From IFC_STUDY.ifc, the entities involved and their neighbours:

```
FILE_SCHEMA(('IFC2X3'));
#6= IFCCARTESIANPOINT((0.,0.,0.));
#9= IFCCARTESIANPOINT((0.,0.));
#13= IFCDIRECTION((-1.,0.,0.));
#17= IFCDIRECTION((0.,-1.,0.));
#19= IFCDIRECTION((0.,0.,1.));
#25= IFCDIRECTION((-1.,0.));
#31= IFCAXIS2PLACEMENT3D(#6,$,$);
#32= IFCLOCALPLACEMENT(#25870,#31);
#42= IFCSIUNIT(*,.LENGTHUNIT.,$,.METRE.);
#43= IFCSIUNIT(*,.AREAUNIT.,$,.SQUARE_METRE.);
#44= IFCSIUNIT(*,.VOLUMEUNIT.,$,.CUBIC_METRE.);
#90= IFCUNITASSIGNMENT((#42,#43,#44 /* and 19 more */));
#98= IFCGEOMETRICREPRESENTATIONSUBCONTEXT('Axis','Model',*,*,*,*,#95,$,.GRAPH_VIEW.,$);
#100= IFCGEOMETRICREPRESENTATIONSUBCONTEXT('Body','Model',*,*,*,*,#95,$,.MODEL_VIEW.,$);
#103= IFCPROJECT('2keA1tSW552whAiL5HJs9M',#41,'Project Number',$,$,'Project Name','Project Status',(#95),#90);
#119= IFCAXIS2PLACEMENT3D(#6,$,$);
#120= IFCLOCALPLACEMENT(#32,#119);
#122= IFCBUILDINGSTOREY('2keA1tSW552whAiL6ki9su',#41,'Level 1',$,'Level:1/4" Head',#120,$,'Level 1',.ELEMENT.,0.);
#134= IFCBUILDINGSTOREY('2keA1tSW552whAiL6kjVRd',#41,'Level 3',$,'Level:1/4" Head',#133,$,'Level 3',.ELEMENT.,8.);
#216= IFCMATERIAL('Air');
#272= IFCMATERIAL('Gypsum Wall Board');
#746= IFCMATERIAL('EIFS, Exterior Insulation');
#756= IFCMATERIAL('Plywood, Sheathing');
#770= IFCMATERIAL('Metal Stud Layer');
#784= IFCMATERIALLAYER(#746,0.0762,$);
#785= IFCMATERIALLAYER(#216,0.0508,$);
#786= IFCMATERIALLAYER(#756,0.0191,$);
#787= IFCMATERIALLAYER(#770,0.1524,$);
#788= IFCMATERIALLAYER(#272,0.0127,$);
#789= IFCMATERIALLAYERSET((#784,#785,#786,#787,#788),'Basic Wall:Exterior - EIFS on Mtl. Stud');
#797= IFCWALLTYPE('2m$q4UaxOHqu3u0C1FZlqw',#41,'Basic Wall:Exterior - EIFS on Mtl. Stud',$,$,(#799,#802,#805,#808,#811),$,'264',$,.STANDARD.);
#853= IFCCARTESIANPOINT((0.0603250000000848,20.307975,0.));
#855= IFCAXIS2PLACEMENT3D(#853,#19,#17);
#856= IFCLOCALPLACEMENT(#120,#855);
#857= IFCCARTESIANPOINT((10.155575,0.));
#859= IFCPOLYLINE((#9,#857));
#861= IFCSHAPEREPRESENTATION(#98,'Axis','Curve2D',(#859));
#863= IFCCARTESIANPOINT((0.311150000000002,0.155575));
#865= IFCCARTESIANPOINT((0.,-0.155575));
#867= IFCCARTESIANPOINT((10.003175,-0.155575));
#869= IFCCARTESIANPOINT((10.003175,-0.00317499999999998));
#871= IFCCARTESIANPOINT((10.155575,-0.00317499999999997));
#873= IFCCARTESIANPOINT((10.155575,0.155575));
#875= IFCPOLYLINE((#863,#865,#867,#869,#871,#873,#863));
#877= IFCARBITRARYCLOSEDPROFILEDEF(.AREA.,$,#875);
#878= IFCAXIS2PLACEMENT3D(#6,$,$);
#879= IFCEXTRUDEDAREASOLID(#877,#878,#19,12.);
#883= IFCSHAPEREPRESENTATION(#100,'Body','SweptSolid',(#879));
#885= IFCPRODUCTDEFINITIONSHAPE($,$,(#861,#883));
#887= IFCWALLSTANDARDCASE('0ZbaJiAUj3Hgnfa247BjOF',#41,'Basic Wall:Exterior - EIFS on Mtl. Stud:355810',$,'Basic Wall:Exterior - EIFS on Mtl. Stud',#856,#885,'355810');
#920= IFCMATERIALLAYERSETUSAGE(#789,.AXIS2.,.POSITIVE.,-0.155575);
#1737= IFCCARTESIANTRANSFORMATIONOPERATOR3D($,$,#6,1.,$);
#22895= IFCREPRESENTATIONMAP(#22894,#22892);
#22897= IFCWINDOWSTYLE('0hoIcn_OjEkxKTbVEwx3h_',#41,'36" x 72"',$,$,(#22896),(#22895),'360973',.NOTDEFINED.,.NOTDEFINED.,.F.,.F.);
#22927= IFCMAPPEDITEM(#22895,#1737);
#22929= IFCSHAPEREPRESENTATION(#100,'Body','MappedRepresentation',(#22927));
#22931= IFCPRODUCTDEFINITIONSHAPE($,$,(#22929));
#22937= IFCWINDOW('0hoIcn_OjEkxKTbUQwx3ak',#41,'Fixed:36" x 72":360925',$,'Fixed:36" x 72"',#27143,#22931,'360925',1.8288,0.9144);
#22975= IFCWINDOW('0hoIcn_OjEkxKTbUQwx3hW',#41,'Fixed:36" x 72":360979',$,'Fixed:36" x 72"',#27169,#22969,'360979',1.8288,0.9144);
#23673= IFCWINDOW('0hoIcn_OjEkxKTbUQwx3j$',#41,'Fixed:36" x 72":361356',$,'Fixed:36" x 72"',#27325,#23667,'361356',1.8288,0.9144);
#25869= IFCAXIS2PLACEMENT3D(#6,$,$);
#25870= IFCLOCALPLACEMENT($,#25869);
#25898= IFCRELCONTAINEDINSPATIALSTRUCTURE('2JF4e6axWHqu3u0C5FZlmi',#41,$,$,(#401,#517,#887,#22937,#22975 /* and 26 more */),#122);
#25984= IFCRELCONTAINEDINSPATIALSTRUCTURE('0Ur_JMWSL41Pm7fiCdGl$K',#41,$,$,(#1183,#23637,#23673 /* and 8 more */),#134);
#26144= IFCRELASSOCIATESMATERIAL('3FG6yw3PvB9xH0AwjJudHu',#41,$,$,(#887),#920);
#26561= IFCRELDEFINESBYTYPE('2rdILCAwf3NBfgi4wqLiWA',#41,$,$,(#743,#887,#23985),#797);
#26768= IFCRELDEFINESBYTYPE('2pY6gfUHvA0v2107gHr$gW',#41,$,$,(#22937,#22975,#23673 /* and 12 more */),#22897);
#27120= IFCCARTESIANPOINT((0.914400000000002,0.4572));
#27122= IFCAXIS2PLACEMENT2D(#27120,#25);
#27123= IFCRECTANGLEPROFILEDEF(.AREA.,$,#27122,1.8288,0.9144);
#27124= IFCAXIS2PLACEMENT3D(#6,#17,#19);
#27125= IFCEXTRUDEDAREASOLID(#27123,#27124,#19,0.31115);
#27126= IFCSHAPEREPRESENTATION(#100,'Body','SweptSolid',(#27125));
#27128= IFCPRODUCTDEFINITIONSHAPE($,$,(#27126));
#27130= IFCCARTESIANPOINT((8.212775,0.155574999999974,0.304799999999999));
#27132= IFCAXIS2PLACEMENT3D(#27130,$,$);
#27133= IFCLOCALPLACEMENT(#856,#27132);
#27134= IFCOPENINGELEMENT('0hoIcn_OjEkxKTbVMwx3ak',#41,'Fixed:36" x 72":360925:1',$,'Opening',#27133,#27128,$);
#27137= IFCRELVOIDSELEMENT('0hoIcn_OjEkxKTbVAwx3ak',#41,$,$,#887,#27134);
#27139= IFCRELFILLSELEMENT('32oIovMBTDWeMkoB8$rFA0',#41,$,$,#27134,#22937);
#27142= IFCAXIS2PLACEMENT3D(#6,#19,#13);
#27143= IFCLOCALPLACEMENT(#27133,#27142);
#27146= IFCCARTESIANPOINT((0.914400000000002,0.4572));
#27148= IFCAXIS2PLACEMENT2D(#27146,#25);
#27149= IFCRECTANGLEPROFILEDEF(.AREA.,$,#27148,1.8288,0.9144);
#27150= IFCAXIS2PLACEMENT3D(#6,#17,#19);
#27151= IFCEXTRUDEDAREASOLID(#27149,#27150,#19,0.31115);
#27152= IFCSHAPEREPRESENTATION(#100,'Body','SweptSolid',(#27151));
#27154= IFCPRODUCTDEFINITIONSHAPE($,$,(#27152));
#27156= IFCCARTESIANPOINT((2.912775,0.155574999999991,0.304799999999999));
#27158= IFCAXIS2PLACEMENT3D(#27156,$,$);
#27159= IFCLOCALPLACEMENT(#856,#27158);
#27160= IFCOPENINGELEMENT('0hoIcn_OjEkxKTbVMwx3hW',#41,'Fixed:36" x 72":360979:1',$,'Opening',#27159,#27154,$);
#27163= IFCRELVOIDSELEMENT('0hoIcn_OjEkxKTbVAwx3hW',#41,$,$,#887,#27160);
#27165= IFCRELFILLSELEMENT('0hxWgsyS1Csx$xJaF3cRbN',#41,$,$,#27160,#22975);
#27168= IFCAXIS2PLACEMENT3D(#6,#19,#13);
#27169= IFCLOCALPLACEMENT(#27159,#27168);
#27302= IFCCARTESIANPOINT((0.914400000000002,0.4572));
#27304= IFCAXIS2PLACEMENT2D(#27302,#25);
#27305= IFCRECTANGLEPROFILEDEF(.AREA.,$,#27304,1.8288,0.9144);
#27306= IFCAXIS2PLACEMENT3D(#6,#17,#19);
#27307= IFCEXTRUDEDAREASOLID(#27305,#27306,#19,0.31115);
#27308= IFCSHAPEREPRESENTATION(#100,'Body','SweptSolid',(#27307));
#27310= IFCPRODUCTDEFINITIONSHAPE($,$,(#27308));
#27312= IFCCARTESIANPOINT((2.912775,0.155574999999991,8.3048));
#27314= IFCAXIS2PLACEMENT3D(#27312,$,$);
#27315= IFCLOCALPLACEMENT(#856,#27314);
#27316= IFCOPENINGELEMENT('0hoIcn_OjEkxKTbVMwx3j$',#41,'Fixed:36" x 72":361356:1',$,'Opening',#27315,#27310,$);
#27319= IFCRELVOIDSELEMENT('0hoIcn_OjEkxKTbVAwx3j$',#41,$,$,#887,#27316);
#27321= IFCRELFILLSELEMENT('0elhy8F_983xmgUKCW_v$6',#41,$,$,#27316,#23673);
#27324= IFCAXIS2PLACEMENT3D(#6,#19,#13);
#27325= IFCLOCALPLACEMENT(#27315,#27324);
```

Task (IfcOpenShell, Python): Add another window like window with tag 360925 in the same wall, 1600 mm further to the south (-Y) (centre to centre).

```python
import ifcopenshell
import ifcopenshell.api.feature
import ifcopenshell.api.geometry
import ifcopenshell.api.root
import ifcopenshell.geom
import ifcopenshell.util.element
import ifcopenshell.util.placement
import ifcopenshell.util.shape

model = ifcopenshell.open("IFC_STUDY.ifc")
settings = ifcopenshell.geom.settings()


def volume(element):
    """Net volume in cubic metres, openings subtracted."""
    shape = ifcopenshell.geom.create_shape(settings, element)
    return ifcopenshell.util.shape.get_volume(shape.geometry)


def reuse_history(source, copy):
    """copy_class also copies each property set's owner history, people and application; keep the originals."""
    for rel in copy.IsDefinedBy:
        if rel.is_a("IfcRelDefinesByProperties") and (history := rel.RelatingPropertyDefinition.OwnerHistory):
            rel.RelatingPropertyDefinition.OwnerHistory = source.OwnerHistory
            ifcopenshell.util.element.remove_deep2(model, history)


window = model.by_guid("0hoIcn_OjEkxKTbUQwx3ak")
opening = window.FillsVoids[0].RelatingOpeningElement
wall = opening.VoidsElements[0].RelatingBuildingElement
before = volume(wall)
shift = ifcopenshell.util.placement.get_local_placement(wall.ObjectPlacement)[:3, 0] * 1.6

# copy_class copies the void relationship, type, container and properties, but no geometry.
new_opening = ifcopenshell.api.root.copy_class(model, product=opening)
new_opening.Representation = ifcopenshell.util.element.copy_deep(
    model, opening.Representation, exclude=["IfcGeometricRepresentationContext", "IfcRepresentationMap"]
)
new_opening.Name = 'Fixed:36" x 72"'
new_window = ifcopenshell.api.root.copy_class(model, product=window)
new_window.Representation = ifcopenshell.util.element.copy_deep(
    model, window.Representation, exclude=["IfcGeometricRepresentationContext", "IfcRepresentationMap"]
)
new_window.Name = 'Fixed:36" x 72"'
new_window.Tag = None
reuse_history(window, new_window)
fills = ifcopenshell.api.feature.add_filling(model, opening=new_opening, element=new_window)
fills.OwnerHistory = new_window.OwnerHistory  # required in IFC2X3

for old, new in ((opening, new_opening), (window, new_window)):
    matrix = ifcopenshell.util.placement.get_local_placement(old.ObjectPlacement)
    matrix[:3, 3] += shift
    ifcopenshell.api.geometry.edit_object_placement(model, product=new, matrix=matrix, is_si=False)

after = volume(wall)

print(f"wall volume {before:.3f} -> {after:.3f} m3")

model.write("IFC_STUDY_rev.ifc")
```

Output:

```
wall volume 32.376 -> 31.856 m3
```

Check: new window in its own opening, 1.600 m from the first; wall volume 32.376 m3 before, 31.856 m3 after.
